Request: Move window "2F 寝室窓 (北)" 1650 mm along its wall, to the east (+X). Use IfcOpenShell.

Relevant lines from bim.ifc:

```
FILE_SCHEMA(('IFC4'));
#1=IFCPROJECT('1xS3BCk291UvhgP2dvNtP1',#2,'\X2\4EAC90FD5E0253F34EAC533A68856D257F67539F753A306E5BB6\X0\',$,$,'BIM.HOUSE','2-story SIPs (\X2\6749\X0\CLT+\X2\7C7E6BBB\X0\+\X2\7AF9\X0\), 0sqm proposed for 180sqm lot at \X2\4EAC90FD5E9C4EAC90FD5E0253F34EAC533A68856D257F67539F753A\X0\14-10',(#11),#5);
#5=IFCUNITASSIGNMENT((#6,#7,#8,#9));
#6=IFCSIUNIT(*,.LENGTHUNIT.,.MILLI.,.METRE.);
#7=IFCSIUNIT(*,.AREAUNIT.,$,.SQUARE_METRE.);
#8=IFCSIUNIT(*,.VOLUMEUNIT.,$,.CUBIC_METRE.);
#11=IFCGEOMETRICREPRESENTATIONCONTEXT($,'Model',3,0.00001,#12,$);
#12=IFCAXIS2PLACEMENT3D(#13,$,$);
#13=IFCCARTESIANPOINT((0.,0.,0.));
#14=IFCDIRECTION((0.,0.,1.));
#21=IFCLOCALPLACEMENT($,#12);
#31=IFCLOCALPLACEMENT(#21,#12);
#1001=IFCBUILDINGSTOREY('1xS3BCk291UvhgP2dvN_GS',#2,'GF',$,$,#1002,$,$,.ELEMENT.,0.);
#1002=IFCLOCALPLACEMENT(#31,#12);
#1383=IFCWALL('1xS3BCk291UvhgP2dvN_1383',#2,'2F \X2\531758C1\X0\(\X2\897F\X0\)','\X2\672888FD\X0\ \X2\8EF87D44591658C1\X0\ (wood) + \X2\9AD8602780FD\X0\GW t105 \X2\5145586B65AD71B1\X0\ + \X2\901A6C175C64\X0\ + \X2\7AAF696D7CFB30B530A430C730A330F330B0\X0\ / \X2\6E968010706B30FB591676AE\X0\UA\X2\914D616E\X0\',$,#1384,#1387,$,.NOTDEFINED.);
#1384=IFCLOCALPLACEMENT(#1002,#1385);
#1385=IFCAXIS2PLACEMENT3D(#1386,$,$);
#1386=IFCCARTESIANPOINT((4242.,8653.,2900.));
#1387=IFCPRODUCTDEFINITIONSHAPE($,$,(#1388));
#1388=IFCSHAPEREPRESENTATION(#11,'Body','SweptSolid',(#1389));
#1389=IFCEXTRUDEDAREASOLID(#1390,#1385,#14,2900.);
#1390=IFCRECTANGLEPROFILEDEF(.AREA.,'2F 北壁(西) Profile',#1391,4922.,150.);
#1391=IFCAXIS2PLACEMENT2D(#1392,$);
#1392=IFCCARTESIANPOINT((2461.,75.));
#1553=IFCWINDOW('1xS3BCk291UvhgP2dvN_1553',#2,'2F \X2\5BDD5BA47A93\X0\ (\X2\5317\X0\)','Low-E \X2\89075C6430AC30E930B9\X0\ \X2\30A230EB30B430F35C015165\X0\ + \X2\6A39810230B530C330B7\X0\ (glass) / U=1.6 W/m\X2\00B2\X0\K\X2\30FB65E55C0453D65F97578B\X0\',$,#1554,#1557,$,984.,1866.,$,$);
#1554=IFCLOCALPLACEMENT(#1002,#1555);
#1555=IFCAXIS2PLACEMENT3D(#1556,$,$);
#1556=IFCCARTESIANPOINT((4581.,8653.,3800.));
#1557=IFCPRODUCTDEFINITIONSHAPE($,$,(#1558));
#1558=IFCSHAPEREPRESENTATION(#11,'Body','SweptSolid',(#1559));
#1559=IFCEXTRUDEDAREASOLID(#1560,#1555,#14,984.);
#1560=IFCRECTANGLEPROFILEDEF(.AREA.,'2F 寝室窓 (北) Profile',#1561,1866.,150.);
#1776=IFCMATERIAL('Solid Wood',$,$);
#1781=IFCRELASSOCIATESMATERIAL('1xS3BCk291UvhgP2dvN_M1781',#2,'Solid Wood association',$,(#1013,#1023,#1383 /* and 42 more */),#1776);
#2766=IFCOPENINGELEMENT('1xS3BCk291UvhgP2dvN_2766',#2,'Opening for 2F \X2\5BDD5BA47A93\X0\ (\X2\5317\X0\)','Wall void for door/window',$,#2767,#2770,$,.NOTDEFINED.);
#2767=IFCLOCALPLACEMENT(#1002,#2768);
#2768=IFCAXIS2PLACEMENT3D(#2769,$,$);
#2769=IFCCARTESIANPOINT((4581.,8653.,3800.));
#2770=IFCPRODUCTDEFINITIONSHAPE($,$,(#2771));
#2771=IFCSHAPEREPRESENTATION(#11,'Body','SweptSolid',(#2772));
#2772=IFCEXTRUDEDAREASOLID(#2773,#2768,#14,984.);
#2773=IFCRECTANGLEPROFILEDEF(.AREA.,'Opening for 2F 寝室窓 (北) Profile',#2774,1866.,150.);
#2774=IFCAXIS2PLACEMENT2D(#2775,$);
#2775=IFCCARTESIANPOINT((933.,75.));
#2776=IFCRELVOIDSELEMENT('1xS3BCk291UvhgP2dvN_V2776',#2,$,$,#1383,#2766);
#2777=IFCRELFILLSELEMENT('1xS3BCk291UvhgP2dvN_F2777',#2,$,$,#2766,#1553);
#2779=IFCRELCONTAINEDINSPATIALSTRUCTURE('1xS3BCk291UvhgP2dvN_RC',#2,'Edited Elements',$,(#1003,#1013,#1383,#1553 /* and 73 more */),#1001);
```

```python
import ifcopenshell
import ifcopenshell.api.geometry
import ifcopenshell.util.placement
import ifcopenshell.util.unit

model = ifcopenshell.open("bim.ifc")
unit_scale = ifcopenshell.util.unit.calculate_unit_scale(model)

window = model.by_guid("1xS3BCk291UvhgP2dvN_1553")
opening = window.FillsVoids[0].RelatingOpeningElement
wall = opening.VoidsElements[0].RelatingBuildingElement

wall_matrix = ifcopenshell.util.placement.get_local_placement(wall.ObjectPlacement)
shift = wall_matrix[:3, 0] * 1.65 / unit_scale
before = ifcopenshell.util.placement.get_local_placement(window.ObjectPlacement)[:3, 3].copy()

# The window is not placed relative to its opening, so move both.
for product in (opening, window):
    matrix = ifcopenshell.util.placement.get_local_placement(product.ObjectPlacement)
    matrix[:3, 3] += shift
    ifcopenshell.api.geometry.edit_object_placement(model, product=product, matrix=matrix, is_si=False)

after = ifcopenshell.util.placement.get_local_placement(window.ObjectPlacement)[:3, 3]
print("window moved by", (after - before).round(3) + 0.0)

model.write("bim_updated.ifc")
```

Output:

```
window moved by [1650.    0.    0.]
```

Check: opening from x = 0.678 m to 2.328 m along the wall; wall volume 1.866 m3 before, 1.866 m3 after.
